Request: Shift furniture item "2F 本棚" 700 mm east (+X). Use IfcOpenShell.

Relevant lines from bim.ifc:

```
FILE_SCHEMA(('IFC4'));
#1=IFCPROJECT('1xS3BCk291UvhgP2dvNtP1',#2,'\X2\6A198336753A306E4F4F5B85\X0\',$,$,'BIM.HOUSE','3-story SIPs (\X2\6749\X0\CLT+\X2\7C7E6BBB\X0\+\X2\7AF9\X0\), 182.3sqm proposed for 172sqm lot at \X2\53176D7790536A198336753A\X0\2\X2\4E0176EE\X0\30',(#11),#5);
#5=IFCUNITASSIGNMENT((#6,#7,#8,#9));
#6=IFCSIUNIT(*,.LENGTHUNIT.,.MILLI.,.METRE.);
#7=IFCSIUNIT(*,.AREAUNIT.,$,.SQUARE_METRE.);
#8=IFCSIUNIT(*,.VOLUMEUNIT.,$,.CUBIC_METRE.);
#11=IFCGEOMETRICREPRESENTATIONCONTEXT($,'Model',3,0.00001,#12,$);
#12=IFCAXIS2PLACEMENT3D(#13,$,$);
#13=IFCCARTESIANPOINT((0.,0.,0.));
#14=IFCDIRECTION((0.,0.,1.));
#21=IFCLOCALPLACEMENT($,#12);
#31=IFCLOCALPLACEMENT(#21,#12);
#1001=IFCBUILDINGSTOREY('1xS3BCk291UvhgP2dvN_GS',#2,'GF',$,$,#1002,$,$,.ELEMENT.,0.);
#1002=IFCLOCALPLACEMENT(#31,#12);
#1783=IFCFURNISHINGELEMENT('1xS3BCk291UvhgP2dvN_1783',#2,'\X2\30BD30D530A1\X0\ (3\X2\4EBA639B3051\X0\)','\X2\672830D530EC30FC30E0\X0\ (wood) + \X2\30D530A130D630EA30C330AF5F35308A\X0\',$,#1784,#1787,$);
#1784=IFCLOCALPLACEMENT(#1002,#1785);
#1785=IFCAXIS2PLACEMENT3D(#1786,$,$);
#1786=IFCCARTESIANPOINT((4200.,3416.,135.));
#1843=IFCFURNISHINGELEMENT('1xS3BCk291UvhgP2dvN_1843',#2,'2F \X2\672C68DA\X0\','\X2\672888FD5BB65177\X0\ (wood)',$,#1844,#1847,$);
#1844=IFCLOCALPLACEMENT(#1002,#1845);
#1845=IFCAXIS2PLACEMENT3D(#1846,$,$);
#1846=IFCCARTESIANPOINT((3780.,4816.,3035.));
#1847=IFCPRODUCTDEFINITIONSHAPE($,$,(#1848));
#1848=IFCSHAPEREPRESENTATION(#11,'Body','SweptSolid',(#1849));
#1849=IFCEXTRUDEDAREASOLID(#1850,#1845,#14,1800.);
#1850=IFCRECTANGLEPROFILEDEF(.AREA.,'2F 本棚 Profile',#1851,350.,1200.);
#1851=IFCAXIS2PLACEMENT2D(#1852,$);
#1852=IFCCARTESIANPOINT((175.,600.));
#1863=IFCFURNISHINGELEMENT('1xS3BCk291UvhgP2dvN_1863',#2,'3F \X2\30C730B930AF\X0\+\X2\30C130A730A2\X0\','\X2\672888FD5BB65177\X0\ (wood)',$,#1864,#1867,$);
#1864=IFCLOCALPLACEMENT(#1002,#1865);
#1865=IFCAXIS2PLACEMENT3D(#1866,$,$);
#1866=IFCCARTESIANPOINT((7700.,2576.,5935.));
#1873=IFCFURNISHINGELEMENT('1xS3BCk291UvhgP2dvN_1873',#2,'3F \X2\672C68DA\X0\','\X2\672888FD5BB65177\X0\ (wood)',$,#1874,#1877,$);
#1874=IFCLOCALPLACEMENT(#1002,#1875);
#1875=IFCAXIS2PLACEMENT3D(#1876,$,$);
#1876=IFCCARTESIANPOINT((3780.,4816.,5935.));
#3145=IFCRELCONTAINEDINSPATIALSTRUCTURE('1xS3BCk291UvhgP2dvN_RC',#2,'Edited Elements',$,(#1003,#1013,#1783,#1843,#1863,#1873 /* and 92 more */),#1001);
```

```python
import ifcopenshell
import ifcopenshell.api.geometry
import ifcopenshell.util.placement

model = ifcopenshell.open("bim.ifc")

item = model.by_id(1843)
matrix = ifcopenshell.util.placement.get_local_placement(item.ObjectPlacement)
matrix[0, 3] += 700.0
ifcopenshell.api.geometry.edit_object_placement(model, product=item, matrix=matrix, is_si=False)

print(ifcopenshell.util.placement.get_local_placement(item.ObjectPlacement).round(3) + 0.0)

model.write("bim_updated.ifc")
```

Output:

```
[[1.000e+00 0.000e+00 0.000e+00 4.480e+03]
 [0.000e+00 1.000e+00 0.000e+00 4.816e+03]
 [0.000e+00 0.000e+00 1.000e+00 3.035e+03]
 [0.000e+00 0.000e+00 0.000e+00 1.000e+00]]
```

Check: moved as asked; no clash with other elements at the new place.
